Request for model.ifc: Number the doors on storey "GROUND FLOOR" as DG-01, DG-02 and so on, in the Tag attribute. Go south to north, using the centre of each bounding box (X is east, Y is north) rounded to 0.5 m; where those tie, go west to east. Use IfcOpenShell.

First a look at what the model holds.

```python
import ifcopenshell
import ifcopenshell.util.element
import ifcopenshell.util.placement

model = ifcopenshell.open("model.ifc")
print(model.schema)
storey = next(s for s in model.by_type("IfcBuildingStorey") if s.Name == "GROUND FLOOR")
doors = [e for e in ifcopenshell.util.element.get_decomposition(storey) if e.is_a("IfcDoor")]
for e in sorted(doors, key=lambda e: e.id()):
    origin = ifcopenshell.util.placement.get_local_placement(e.ObjectPlacement)[:3, 3]
    print(e.id(), e.Tag, e.Name, origin.round(2) + 0.0, sep=" | ")
```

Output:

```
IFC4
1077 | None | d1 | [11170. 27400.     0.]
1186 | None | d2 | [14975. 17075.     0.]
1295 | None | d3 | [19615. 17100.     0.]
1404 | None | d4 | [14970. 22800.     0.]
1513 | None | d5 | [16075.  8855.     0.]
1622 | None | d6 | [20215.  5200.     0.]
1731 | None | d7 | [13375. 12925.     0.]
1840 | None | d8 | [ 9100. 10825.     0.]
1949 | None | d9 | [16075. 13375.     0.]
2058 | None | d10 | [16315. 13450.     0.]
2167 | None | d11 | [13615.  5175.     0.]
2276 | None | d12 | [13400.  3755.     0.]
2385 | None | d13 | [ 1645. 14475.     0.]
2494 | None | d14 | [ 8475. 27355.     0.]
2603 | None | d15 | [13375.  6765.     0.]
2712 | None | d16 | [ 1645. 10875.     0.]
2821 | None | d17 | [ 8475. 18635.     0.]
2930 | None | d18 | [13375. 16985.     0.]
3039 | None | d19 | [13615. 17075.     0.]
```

```python
import ifcopenshell
import ifcopenshell.geom
import ifcopenshell.util.element
import ifcopenshell.util.shape

model = ifcopenshell.open("model.ifc")
settings = ifcopenshell.geom.settings()
settings.set("use-world-coords", True)


def centre(element):
    shape = ifcopenshell.geom.create_shape(settings, element)
    return ifcopenshell.util.shape.get_bbox_centroid(shape.geometry)


storey = next(s for s in model.by_type("IfcBuildingStorey") if s.Name == "GROUND FLOOR")
doors = [e for e in ifcopenshell.util.element.get_decomposition(storey) if e.is_a("IfcDoor")]

# Insertion points can sit at a corner or the storey origin, so sort by the geometry (in metres).
centres = {e: centre(e) for e in doors}
doors.sort(key=lambda e: (round(centres[e][1] / 0.5), centres[e][0]))

for i, e in enumerate(doors, start=1):
    number = f"DG-{i:02d}"
    e.Tag = number
    print(e.id(), number)

model.write("model_v2.ifc")
```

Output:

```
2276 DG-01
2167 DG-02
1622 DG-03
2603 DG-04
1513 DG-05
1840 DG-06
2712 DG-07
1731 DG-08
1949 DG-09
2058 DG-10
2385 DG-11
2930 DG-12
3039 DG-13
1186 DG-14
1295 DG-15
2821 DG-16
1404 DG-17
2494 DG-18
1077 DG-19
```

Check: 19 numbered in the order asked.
